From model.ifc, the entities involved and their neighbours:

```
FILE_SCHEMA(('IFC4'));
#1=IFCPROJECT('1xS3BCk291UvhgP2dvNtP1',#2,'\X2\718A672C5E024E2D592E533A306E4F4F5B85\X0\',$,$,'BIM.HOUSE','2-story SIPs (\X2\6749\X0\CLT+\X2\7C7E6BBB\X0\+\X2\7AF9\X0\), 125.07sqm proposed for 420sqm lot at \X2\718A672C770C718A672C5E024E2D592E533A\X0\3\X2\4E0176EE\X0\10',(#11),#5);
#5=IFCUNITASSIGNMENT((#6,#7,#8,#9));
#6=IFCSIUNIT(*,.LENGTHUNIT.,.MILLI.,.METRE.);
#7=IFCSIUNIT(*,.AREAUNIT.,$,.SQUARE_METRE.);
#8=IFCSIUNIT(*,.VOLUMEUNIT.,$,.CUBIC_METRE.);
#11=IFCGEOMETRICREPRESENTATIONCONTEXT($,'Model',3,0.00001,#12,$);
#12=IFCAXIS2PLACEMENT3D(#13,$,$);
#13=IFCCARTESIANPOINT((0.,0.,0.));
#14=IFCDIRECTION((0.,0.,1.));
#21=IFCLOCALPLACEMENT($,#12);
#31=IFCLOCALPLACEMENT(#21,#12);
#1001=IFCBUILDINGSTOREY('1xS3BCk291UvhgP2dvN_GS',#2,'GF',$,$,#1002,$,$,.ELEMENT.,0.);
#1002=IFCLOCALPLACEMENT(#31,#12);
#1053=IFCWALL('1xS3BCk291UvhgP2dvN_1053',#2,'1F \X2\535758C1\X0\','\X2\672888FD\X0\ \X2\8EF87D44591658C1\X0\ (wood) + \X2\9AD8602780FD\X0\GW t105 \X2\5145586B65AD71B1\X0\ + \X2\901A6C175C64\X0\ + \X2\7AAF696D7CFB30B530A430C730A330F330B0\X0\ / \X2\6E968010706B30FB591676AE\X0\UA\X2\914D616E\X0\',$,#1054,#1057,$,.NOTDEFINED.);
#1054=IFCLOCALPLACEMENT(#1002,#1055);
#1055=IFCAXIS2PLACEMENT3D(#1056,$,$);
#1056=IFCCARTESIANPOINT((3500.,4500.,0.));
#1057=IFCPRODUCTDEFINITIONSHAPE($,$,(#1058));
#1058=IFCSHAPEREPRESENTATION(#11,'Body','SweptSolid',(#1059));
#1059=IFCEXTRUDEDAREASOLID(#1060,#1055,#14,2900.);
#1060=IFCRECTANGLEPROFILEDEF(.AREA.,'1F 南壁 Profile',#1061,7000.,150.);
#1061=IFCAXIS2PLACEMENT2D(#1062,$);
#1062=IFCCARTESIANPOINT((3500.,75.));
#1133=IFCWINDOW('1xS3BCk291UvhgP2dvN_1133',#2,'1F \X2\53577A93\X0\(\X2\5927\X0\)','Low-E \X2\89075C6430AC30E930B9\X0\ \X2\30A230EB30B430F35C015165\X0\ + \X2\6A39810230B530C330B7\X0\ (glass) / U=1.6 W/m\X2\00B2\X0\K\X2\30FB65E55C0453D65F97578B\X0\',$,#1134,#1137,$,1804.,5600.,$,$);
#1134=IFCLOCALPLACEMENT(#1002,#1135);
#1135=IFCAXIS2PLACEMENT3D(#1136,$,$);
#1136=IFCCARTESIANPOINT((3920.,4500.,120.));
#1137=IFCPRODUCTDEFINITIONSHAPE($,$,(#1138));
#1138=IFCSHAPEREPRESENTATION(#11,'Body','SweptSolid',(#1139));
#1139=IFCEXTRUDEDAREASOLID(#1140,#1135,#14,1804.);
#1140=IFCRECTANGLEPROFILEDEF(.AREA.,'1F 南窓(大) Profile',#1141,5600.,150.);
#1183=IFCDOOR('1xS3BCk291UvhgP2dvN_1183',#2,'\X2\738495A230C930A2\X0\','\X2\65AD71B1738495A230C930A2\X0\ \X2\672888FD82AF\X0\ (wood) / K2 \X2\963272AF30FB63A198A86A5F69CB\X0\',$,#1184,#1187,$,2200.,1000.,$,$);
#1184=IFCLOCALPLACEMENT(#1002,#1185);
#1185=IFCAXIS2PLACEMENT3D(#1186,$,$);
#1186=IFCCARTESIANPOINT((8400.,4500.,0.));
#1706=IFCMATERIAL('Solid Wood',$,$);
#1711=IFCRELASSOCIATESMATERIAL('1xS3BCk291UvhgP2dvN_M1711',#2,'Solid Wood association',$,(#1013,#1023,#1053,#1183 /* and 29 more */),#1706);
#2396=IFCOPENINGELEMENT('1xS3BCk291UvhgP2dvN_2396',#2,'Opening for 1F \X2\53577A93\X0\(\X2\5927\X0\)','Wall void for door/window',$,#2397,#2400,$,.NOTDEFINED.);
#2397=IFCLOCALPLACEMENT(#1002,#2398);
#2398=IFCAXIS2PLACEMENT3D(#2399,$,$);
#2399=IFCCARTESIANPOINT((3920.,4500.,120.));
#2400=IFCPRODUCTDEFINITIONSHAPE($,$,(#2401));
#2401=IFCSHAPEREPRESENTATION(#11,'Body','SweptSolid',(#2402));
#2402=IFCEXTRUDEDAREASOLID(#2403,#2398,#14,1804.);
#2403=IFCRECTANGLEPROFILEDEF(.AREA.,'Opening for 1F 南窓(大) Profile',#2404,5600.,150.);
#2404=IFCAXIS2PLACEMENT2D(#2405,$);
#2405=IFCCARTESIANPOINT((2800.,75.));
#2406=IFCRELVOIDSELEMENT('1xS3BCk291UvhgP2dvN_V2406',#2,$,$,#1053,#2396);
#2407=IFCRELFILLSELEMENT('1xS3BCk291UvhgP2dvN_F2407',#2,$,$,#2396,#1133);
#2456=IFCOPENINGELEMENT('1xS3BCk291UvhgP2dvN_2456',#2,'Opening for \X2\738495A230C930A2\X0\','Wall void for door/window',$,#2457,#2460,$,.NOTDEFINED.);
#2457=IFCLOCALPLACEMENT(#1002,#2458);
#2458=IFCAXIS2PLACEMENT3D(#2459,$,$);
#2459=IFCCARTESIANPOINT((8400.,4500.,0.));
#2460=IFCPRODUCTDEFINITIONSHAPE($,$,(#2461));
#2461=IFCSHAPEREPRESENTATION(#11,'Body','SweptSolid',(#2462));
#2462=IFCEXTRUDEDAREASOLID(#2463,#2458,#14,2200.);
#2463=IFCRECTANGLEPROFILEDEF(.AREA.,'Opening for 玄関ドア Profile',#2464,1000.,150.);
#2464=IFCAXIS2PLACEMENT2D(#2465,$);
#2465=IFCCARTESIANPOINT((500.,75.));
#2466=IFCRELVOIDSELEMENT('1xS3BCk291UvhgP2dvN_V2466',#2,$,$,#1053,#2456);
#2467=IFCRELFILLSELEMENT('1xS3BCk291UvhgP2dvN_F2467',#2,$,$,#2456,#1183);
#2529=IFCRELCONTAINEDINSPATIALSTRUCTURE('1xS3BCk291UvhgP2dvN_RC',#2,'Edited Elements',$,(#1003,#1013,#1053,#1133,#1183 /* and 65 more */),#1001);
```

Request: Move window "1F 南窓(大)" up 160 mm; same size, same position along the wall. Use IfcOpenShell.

```python
import numpy as np
import ifcopenshell
import ifcopenshell.api.geometry
import ifcopenshell.util.placement
import ifcopenshell.util.unit

model = ifcopenshell.open("model.ifc")
unit_scale = ifcopenshell.util.unit.calculate_unit_scale(model)

window = model.by_id(1133)
opening = window.FillsVoids[0].RelatingOpeningElement
dz = 0.16 / unit_scale

shift = np.array([0.0, 0.0, dz])
# The window is not placed relative to its opening, so move both.
for product in (opening, window):
    matrix = ifcopenshell.util.placement.get_local_placement(product.ObjectPlacement)
    matrix[:3, 3] += shift
    ifcopenshell.api.geometry.edit_object_placement(model, product=product, matrix=matrix, is_si=False)

print(f"moved by {dz * unit_scale:+.3f} m")

model.write("model_edited.ifc")
```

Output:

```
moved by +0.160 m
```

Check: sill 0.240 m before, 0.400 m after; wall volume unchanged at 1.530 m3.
